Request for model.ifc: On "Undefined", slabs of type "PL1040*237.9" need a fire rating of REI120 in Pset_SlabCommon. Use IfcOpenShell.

First a look at what the model holds.

```python
import ifcopenshell
import ifcopenshell.util.element

model = ifcopenshell.open("model.ifc")
print(model.schema)
storey = next(s for s in model.by_type("IfcBuildingStorey") if s.Name == "Undefined")
slabs = [e for e in ifcopenshell.util.element.get_decomposition(storey) if e.is_a("IfcSlab")]
seen = {}
for e in slabs:
    element_type = ifcopenshell.util.element.get_type(e)
    key = (element_type.Name if element_type != e and element_type else None, ifcopenshell.util.element.get_pset(e, "Pset_SlabCommon", "FireRating"))
    seen[key] = seen.get(key, 0) + 1
for (name, value), count in sorted(seen.items(), key=str):
    print(count, "x", name, "|", value)
```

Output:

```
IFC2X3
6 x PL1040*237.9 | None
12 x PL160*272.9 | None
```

```python
import ifcopenshell
import ifcopenshell.api.pset
import ifcopenshell.util.element

model = ifcopenshell.open("model.ifc")

storey = next(s for s in model.by_type("IfcBuildingStorey") if s.Name == "Undefined")
slabs = [e for e in ifcopenshell.util.element.get_decomposition(storey) if e.is_a("IfcSlab")]

count = 0
for e in slabs:
    element_type = ifcopenshell.util.element.get_type(e)
    if element_type in (None, e) or element_type.Name != "PL1040*237.9":
        continue
    # add_pset returns the element's existing set when there is one.
    pset = ifcopenshell.api.pset.add_pset(model, product=e, name="Pset_SlabCommon")
    ifcopenshell.api.pset.edit_pset(model, pset=pset, properties={"FireRating": "REI120"})
    count += 1

print(count, "slabs updated")

model.write("model_edited.ifc")
```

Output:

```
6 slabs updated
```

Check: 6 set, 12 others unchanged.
